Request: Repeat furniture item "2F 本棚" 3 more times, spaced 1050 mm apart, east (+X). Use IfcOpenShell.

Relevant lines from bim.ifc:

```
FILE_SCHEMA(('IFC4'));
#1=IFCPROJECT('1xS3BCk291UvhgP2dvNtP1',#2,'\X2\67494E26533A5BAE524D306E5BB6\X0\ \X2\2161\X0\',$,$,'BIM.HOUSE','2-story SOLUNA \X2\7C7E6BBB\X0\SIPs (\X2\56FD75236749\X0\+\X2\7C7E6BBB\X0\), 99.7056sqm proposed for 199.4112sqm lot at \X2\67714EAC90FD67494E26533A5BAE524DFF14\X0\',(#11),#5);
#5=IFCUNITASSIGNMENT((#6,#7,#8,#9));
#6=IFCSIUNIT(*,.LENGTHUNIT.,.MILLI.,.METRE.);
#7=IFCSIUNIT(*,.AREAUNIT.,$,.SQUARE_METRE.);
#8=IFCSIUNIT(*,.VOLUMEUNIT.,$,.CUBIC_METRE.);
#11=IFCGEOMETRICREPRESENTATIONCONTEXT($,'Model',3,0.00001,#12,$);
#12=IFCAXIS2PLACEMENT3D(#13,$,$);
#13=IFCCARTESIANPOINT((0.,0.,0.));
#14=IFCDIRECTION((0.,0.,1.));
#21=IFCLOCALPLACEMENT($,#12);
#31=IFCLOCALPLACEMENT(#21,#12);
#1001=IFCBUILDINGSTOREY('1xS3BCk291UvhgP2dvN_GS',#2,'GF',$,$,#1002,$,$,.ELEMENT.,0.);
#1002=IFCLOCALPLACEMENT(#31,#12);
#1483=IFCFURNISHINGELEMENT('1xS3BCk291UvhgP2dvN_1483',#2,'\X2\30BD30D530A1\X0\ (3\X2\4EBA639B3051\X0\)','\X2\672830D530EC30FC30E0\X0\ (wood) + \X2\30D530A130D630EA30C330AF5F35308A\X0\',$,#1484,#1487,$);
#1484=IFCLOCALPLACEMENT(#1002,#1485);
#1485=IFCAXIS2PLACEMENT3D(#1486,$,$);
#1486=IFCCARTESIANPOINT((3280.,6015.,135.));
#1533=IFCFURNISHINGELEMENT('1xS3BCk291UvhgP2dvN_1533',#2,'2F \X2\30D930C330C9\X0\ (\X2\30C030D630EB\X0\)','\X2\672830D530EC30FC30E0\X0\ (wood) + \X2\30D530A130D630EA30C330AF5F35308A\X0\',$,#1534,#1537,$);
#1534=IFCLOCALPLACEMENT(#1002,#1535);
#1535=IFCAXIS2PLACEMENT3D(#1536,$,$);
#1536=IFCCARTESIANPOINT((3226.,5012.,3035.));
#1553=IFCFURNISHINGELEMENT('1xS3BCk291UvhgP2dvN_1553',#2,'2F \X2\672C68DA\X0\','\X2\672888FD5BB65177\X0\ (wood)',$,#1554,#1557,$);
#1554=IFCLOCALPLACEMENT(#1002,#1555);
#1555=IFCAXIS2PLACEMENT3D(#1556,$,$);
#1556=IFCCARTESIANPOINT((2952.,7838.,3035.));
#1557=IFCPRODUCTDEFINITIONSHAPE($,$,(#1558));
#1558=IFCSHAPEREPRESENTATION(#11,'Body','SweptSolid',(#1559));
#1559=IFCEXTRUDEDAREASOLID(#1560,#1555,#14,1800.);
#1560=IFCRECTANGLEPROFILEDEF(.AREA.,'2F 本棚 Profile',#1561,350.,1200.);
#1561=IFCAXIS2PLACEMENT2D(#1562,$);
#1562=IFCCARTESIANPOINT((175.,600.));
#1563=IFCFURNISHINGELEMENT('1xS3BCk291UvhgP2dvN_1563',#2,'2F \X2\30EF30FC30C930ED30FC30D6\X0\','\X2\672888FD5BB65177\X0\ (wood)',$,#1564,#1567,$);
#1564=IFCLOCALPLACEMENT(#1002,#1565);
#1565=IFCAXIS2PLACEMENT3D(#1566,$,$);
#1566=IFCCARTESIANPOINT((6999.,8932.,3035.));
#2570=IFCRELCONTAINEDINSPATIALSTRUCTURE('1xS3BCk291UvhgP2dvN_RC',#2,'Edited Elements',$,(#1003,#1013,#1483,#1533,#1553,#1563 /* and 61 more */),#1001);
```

```python
import numpy as np
import ifcopenshell
import ifcopenshell.api.geometry
import ifcopenshell.api.root
import ifcopenshell.util.element
import ifcopenshell.util.placement
import ifcopenshell.util.unit

model = ifcopenshell.open("bim.ifc")
unit_scale = ifcopenshell.util.unit.calculate_unit_scale(model)


def reuse_history(source, copy):
    """copy_class also copies each property set's owner history, people and application; keep the originals."""
    for rel in copy.IsDefinedBy:
        if rel.is_a("IfcRelDefinesByProperties") and (history := rel.RelatingPropertyDefinition.OwnerHistory):
            rel.RelatingPropertyDefinition.OwnerHistory = source.OwnerHistory
            ifcopenshell.util.element.remove_deep2(model, history)


source = model.by_guid("1xS3BCk291UvhgP2dvN_1553")
base = ifcopenshell.util.placement.get_local_placement(source.ObjectPlacement)
step = np.array([1.0, 0.0, 0.0]) * 1.05 / unit_scale

for i in range(1, 4):
    copy = ifcopenshell.api.root.copy_class(model, product=source)
    copy.Representation = ifcopenshell.util.element.copy_deep(
        model, source.Representation, exclude=["IfcGeometricRepresentationContext", "IfcRepresentationMap"]
    )
    reuse_history(source, copy)
    matrix = base.copy()
    matrix[:3, 3] += i * step
    print("added at", matrix[:3, 3].round(3) + 0.0)
    ifcopenshell.api.geometry.edit_object_placement(model, product=copy, matrix=matrix, is_si=False)

model.write("bim_updated.ifc")
```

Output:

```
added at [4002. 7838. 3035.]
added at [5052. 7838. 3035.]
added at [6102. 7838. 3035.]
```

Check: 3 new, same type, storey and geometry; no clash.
